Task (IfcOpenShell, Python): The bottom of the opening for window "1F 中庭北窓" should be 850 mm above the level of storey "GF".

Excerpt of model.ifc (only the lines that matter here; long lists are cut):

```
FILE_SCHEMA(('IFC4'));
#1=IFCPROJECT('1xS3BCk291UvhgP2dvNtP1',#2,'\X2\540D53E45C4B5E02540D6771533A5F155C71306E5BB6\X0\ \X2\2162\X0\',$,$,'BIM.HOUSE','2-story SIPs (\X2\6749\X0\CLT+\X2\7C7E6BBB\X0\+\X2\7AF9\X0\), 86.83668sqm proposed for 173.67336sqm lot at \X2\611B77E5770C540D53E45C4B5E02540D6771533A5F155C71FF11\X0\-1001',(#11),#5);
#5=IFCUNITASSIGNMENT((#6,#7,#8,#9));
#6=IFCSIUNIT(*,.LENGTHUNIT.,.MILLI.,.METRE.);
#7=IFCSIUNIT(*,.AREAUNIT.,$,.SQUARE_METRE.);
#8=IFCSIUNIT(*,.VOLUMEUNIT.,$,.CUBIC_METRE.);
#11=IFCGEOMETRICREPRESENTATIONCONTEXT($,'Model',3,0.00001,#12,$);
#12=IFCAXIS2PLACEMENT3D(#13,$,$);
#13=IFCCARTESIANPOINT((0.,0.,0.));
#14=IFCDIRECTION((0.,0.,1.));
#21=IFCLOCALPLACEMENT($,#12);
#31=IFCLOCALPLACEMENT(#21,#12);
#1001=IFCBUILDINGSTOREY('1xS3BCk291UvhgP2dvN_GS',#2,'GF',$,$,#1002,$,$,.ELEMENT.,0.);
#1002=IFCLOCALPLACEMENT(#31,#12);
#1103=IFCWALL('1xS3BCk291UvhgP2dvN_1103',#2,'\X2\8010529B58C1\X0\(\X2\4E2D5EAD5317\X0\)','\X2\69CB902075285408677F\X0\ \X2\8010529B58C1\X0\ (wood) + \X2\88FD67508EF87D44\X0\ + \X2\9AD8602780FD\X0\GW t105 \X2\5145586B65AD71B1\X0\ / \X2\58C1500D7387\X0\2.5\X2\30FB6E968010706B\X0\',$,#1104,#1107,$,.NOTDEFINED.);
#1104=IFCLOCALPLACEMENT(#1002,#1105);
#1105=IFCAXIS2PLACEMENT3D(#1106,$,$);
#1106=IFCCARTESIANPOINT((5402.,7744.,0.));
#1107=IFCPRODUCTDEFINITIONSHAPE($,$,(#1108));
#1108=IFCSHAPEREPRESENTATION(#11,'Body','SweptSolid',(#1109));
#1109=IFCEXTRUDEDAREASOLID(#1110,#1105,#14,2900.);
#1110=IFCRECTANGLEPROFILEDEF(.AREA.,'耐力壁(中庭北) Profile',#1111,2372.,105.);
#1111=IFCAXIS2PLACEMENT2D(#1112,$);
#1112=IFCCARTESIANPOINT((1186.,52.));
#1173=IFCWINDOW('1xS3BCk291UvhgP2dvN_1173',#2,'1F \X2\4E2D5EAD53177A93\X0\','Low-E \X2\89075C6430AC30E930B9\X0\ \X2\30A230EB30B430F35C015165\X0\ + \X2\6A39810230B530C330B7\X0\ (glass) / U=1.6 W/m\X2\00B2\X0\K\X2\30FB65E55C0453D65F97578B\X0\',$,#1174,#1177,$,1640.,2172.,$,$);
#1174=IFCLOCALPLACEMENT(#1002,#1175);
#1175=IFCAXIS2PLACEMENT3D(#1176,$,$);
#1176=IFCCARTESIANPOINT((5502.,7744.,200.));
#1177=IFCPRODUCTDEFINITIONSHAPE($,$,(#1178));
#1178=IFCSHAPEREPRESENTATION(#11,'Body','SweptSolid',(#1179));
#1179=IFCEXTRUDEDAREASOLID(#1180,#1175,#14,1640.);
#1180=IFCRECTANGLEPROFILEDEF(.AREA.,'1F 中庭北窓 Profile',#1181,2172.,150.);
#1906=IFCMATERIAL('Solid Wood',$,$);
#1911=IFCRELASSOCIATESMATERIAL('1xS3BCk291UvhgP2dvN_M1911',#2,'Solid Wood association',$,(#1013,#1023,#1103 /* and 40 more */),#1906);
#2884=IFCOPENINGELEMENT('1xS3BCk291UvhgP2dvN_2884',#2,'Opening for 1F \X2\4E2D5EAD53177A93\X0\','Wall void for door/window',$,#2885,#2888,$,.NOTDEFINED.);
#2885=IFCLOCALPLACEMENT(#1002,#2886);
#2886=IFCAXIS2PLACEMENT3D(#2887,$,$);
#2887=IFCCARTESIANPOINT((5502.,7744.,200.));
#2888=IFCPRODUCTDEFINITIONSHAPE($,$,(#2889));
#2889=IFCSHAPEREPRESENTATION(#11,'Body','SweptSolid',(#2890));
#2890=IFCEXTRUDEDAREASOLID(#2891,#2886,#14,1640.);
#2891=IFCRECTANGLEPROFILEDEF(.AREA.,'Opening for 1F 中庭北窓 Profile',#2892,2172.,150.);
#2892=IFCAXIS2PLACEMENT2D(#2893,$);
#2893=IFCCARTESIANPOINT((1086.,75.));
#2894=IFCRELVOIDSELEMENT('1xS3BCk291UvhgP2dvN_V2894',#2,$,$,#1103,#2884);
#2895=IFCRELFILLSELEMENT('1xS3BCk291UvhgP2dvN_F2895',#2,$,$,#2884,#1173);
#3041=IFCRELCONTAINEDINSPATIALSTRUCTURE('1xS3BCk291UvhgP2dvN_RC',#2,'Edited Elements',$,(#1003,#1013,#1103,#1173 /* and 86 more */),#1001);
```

```python
import numpy as np
import ifcopenshell
import ifcopenshell.api.geometry
import ifcopenshell.geom
import ifcopenshell.util.element
import ifcopenshell.util.placement
import ifcopenshell.util.shape
import ifcopenshell.util.unit

model = ifcopenshell.open("model.ifc")
unit_scale = ifcopenshell.util.unit.calculate_unit_scale(model)

window = model.by_guid("1xS3BCk291UvhgP2dvN_1173")
opening = window.FillsVoids[0].RelatingOpeningElement
storey = ifcopenshell.util.element.get_container(window, ifc_class="IfcBuildingStorey")
level = ifcopenshell.util.placement.get_local_placement(storey.ObjectPlacement)[2, 3]

# The opening's origin need not be at the sill, so measure its lowest point.
shape = ifcopenshell.geom.create_shape(ifcopenshell.geom.settings(), opening)
bottom = ifcopenshell.util.shape.get_shape_bottom_elevation(shape, shape.geometry) / unit_scale
dz = level + 0.85 / unit_scale - bottom

shift = np.array([0.0, 0.0, dz])
# The window is not placed relative to its opening, so move both.
for product in (opening, window):
    matrix = ifcopenshell.util.placement.get_local_placement(product.ObjectPlacement)
    matrix[:3, 3] += shift
    ifcopenshell.api.geometry.edit_object_placement(model, product=product, matrix=matrix, is_si=False)

print(f"moved by {dz * unit_scale:+.3f} m")

model.write("model_rev.ifc")
```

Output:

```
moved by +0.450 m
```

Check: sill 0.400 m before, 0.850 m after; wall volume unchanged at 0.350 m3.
